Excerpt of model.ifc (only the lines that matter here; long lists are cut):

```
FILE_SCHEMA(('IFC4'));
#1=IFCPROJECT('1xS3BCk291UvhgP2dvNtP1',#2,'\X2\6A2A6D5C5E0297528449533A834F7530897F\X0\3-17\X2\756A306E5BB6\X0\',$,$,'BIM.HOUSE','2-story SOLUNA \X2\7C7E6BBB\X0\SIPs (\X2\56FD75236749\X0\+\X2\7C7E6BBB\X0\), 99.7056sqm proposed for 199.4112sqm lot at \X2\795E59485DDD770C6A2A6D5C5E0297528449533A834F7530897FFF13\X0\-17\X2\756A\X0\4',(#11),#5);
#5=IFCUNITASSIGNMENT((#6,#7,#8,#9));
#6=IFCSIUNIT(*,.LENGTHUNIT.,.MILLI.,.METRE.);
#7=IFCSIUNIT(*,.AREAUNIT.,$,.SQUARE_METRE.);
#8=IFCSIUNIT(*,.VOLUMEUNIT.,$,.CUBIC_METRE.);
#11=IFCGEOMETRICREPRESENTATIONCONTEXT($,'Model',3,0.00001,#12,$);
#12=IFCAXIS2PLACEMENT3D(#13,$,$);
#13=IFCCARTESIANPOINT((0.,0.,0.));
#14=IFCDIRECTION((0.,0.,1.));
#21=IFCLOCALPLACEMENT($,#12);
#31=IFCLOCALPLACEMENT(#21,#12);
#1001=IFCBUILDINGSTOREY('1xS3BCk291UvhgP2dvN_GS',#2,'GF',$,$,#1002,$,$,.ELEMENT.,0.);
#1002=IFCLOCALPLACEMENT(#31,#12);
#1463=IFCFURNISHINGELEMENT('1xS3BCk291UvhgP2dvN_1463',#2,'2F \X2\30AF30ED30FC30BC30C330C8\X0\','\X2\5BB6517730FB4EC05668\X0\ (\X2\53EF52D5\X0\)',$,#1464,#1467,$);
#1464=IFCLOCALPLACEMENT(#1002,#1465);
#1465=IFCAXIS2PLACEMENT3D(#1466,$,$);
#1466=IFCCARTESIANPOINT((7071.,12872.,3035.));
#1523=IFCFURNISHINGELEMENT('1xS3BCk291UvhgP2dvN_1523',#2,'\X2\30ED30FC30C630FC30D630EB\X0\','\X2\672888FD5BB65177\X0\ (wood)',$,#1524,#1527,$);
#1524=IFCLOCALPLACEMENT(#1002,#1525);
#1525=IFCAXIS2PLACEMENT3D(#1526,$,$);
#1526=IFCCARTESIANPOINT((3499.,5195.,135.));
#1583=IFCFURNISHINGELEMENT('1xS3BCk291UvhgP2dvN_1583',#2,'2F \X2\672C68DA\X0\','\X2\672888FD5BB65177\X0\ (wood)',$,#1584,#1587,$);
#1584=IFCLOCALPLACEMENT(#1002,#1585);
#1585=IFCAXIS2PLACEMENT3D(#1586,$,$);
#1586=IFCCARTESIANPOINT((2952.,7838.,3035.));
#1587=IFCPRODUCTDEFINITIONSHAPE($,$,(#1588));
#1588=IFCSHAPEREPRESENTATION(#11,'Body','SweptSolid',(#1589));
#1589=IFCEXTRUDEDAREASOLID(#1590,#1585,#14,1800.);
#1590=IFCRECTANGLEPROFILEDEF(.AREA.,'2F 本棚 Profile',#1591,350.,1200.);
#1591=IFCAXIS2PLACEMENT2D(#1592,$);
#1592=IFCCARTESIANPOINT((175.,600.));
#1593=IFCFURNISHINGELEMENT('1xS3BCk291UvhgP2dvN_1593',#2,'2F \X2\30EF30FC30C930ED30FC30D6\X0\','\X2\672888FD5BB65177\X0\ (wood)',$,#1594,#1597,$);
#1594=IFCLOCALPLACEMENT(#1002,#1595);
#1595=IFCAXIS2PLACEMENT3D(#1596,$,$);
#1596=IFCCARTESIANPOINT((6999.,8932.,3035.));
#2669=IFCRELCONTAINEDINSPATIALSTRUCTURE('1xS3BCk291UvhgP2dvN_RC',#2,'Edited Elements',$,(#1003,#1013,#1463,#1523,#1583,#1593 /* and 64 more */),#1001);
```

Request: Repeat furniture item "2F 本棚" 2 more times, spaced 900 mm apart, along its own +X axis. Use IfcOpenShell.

```python
import ifcopenshell
import ifcopenshell.api.geometry
import ifcopenshell.api.root
import ifcopenshell.util.element
import ifcopenshell.util.placement
import ifcopenshell.util.unit

model = ifcopenshell.open("model.ifc")
unit_scale = ifcopenshell.util.unit.calculate_unit_scale(model)


def reuse_history(source, copy):
    """copy_class also copies each property set's owner history, people and application; keep the originals."""
    for rel in copy.IsDefinedBy:
        if rel.is_a("IfcRelDefinesByProperties") and (history := rel.RelatingPropertyDefinition.OwnerHistory):
            rel.RelatingPropertyDefinition.OwnerHistory = source.OwnerHistory
            ifcopenshell.util.element.remove_deep2(model, history)


source = model.by_guid("1xS3BCk291UvhgP2dvN_1583")
base = ifcopenshell.util.placement.get_local_placement(source.ObjectPlacement)
step = base[:3, 0] * 0.9 / unit_scale

for i in range(1, 3):
    copy = ifcopenshell.api.root.copy_class(model, product=source)
    copy.Representation = ifcopenshell.util.element.copy_deep(
        model, source.Representation, exclude=["IfcGeometricRepresentationContext", "IfcRepresentationMap"]
    )
    reuse_history(source, copy)
    matrix = base.copy()
    matrix[:3, 3] += i * step
    print("added at", matrix[:3, 3].round(3) + 0.0)
    ifcopenshell.api.geometry.edit_object_placement(model, product=copy, matrix=matrix, is_si=False)

model.write("model_updated.ifc")
```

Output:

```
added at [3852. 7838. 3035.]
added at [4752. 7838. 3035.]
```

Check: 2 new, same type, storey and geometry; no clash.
